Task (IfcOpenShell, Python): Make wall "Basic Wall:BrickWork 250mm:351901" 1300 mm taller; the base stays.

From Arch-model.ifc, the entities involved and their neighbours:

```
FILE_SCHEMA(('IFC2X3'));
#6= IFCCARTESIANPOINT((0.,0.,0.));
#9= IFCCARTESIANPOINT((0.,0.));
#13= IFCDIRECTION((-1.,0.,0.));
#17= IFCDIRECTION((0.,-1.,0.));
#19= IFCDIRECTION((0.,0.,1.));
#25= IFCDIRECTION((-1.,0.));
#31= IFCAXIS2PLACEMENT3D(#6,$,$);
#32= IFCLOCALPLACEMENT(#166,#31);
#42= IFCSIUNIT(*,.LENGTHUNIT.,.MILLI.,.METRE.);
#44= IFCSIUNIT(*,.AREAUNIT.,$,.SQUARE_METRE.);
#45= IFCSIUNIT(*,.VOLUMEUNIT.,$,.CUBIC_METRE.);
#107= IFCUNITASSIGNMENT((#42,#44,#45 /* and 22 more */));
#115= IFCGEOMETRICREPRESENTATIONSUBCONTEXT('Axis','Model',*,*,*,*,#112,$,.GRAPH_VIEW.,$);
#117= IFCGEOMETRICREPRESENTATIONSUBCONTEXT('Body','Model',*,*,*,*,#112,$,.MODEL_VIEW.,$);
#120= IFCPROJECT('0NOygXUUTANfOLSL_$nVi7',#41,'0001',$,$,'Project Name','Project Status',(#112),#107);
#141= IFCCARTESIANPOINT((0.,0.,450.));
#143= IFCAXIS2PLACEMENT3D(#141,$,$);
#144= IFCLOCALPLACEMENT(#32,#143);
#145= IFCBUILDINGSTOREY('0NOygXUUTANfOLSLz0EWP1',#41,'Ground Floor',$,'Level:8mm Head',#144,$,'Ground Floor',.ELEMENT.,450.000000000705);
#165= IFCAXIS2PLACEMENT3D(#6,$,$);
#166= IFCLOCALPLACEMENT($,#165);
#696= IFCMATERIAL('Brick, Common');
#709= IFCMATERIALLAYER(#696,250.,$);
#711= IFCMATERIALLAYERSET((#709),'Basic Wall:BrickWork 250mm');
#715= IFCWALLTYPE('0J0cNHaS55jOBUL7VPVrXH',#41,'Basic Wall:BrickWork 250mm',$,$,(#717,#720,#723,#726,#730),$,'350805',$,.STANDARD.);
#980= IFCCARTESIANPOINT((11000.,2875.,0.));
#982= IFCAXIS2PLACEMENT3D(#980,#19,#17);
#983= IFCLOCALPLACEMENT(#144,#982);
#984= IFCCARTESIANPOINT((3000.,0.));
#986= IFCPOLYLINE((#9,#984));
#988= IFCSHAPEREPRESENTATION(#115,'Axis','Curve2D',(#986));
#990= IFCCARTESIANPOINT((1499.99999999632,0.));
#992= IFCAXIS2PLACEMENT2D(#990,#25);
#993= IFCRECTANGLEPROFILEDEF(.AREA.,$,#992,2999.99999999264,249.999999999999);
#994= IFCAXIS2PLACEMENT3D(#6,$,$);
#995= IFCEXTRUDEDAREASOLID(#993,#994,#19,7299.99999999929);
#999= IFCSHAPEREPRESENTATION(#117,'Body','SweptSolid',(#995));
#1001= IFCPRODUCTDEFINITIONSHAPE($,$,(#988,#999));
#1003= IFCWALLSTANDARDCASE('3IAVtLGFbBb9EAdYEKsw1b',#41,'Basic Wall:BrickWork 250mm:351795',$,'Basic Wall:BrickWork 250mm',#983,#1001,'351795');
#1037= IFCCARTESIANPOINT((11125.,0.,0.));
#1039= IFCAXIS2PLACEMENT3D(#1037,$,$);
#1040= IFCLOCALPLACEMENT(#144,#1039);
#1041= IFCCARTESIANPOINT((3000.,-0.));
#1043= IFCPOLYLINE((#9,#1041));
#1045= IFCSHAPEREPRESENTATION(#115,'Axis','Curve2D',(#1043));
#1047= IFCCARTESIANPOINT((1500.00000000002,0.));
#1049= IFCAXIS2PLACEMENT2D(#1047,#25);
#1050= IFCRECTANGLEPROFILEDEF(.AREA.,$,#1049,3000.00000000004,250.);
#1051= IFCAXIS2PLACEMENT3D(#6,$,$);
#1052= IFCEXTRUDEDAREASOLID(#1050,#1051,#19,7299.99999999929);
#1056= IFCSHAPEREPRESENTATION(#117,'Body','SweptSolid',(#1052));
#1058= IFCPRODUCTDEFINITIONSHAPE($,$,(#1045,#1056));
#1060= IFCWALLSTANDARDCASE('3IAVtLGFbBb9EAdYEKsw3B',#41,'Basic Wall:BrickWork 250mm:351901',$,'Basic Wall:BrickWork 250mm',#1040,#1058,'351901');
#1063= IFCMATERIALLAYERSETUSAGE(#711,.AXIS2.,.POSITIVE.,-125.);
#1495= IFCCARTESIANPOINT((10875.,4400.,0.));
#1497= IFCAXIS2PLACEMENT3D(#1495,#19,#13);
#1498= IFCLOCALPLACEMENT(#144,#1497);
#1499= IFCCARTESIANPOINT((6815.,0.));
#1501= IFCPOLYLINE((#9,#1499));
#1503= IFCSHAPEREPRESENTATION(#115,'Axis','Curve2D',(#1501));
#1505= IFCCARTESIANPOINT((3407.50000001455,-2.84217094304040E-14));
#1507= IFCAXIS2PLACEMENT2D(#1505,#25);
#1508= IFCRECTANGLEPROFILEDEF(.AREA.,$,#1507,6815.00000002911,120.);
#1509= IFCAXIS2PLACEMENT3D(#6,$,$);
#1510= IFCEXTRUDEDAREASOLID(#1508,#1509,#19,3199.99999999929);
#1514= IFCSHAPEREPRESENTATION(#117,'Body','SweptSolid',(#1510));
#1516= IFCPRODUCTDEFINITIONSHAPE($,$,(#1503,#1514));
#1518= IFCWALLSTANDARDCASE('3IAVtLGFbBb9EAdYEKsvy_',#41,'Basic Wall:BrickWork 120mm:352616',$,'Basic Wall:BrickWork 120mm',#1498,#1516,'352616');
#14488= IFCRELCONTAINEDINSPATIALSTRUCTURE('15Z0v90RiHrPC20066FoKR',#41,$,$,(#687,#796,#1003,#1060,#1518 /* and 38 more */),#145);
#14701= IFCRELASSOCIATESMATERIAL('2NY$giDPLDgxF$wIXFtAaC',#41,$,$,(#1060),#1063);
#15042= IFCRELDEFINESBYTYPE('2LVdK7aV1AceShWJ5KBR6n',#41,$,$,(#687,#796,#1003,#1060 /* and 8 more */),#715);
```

```python
import ifcopenshell
import ifcopenshell.geom
import ifcopenshell.util.representation
import ifcopenshell.util.shape

model = ifcopenshell.open("Arch-model.ifc")
settings = ifcopenshell.geom.settings()


def volume(element):
    """Net volume in cubic metres, openings subtracted."""
    shape = ifcopenshell.geom.create_shape(settings, element)
    return ifcopenshell.util.shape.get_volume(shape.geometry)


wall = model.by_guid("3IAVtLGFbBb9EAdYEKsw3B")
before = volume(wall)

body = ifcopenshell.util.representation.get_representation(wall, "Model", "Body")
solid = body.Items[0]
old_height = solid.Depth
solid.Depth += 1300.0
after = volume(wall)

print(f"height {old_height:g} -> {solid.Depth:g}, volume {before:.3f} -> {after:.3f} m3")

model.write("Arch-model_edited.ifc")
```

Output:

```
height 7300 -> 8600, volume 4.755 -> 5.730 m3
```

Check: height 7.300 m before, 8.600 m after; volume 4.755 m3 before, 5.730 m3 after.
